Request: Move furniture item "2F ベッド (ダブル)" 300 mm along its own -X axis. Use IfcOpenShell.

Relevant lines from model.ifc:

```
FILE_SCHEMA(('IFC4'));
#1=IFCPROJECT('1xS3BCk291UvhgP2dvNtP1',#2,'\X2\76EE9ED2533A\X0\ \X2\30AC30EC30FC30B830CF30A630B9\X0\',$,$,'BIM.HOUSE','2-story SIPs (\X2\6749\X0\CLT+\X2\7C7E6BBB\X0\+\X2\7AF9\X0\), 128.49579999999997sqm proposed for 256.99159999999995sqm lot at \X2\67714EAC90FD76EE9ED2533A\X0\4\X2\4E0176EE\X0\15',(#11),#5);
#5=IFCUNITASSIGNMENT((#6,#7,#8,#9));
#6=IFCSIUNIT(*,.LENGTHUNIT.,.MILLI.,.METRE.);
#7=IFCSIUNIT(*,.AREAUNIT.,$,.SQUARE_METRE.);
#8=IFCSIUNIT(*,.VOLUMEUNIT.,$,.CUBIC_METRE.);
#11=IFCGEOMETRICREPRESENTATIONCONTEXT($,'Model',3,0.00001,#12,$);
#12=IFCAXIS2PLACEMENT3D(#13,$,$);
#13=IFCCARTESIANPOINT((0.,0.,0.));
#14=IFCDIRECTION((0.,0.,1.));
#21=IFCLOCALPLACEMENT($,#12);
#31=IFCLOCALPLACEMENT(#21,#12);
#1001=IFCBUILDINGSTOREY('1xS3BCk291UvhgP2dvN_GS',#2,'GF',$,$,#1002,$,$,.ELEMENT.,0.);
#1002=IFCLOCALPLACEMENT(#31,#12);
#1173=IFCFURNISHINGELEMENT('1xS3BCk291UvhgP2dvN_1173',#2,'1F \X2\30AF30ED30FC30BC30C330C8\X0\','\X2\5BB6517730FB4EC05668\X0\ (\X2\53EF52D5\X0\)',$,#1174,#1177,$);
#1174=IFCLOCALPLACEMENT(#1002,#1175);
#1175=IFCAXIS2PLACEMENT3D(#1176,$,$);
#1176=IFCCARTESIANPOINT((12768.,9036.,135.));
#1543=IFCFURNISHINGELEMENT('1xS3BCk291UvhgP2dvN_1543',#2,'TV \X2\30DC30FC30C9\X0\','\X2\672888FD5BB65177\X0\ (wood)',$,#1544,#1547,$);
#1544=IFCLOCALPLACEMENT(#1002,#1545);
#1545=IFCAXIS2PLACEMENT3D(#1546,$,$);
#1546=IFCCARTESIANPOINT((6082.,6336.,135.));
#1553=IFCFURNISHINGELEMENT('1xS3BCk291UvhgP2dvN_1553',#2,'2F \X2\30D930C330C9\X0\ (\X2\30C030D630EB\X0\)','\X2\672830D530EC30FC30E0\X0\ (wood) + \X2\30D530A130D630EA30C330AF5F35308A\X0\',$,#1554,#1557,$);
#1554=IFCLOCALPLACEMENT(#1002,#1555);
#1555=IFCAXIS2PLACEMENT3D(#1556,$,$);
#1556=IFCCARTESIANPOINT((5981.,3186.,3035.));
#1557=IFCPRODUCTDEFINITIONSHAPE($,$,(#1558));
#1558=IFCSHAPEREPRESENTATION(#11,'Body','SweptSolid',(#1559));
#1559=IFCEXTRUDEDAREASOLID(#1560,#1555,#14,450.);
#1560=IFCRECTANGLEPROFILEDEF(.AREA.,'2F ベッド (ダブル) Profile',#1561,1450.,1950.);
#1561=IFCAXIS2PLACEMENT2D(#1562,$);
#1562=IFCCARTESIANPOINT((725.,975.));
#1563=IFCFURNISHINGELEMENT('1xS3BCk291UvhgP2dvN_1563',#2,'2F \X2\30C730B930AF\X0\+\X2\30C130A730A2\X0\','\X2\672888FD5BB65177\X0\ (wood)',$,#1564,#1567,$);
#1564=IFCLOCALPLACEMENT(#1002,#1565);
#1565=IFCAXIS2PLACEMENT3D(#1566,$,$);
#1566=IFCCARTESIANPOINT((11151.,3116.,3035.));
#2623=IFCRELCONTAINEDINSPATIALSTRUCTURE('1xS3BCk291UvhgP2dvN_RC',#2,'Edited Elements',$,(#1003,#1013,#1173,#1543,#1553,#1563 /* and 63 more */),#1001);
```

```python
import ifcopenshell
import ifcopenshell.api.geometry
import ifcopenshell.util.placement

model = ifcopenshell.open("model.ifc")

item = model.by_guid("1xS3BCk291UvhgP2dvN_1553")
matrix = ifcopenshell.util.placement.get_local_placement(item.ObjectPlacement)
matrix[:3, 3] -= matrix[:3, 0] * 300.0
ifcopenshell.api.geometry.edit_object_placement(model, product=item, matrix=matrix, is_si=False)

print(ifcopenshell.util.placement.get_local_placement(item.ObjectPlacement).round(3) + 0.0)

model.write("model_rev.ifc")
```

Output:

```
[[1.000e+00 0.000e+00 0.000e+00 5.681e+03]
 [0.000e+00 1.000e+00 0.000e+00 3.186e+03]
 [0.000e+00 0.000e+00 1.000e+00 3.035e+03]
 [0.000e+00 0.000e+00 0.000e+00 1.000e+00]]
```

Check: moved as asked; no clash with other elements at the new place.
